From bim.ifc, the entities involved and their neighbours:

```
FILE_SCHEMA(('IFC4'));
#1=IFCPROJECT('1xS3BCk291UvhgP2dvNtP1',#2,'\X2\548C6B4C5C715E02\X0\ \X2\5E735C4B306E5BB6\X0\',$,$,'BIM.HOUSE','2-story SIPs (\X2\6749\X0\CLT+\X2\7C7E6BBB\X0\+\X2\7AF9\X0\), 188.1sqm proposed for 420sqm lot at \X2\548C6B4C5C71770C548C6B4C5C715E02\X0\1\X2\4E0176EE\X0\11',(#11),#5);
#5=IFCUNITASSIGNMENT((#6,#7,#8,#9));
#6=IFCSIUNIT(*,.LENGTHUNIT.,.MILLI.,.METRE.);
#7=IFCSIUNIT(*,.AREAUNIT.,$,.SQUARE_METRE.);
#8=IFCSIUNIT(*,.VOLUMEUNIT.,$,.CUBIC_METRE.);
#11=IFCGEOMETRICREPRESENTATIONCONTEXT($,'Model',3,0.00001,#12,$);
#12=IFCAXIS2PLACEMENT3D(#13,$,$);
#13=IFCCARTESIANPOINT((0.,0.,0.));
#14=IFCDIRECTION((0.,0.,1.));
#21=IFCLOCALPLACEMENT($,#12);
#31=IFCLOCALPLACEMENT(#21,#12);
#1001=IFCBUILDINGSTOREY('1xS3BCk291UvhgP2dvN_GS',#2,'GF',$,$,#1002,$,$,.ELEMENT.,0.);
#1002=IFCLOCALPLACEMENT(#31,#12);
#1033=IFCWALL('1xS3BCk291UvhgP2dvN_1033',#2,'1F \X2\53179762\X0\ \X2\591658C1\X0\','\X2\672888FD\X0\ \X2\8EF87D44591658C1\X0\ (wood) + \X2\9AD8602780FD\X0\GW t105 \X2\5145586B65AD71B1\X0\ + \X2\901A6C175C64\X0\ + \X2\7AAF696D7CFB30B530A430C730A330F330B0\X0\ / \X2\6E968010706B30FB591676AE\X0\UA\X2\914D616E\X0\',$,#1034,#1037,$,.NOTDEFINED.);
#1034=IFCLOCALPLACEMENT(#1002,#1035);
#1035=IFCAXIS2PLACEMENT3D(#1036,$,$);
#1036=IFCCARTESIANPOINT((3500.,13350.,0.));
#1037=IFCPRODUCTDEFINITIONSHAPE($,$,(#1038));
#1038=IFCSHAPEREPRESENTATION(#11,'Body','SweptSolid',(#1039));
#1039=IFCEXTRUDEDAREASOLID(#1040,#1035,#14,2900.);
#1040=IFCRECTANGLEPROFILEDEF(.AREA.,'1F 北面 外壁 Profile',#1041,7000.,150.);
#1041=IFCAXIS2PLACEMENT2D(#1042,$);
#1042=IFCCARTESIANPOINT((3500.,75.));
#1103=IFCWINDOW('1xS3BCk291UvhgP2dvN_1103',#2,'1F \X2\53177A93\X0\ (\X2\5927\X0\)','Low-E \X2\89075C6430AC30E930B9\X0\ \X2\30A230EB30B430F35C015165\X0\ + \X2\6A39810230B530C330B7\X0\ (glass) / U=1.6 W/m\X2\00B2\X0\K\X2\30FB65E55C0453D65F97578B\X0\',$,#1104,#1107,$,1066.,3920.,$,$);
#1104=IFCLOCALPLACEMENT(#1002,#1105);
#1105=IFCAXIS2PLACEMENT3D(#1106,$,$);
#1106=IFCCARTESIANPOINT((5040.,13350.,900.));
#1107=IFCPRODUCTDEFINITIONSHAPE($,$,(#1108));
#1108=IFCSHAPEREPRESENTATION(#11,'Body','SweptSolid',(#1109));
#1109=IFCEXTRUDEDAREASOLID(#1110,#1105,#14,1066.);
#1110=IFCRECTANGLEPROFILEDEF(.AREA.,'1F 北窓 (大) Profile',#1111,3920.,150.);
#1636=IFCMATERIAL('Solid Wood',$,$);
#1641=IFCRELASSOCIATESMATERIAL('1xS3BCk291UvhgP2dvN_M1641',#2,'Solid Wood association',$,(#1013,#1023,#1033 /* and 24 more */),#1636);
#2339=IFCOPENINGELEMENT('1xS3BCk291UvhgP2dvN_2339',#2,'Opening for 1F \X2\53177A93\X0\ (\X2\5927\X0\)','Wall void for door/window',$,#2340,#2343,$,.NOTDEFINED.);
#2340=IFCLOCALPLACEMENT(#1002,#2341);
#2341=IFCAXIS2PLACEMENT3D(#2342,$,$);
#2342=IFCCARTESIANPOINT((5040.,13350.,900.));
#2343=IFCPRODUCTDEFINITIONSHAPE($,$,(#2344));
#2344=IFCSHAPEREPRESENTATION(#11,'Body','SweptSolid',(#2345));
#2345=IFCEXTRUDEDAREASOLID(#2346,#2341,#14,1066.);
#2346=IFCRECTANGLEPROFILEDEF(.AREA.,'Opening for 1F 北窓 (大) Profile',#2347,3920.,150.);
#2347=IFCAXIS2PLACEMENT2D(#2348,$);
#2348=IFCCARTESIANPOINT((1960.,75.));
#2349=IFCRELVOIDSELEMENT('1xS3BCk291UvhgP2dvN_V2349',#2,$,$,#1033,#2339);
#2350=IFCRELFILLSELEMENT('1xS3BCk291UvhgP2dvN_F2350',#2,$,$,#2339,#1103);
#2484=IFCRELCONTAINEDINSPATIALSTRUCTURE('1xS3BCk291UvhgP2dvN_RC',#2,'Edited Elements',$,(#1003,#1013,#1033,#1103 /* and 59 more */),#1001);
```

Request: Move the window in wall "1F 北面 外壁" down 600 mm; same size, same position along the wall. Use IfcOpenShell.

```python
import numpy as np
import ifcopenshell
import ifcopenshell.api.geometry
import ifcopenshell.util.placement
import ifcopenshell.util.unit

model = ifcopenshell.open("bim.ifc")
unit_scale = ifcopenshell.util.unit.calculate_unit_scale(model)

window = model.by_guid("1xS3BCk291UvhgP2dvN_1103")
opening = window.FillsVoids[0].RelatingOpeningElement
dz = -0.6 / unit_scale

shift = np.array([0.0, 0.0, dz])
# The window is not placed relative to its opening, so move both.
for product in (opening, window):
    matrix = ifcopenshell.util.placement.get_local_placement(product.ObjectPlacement)
    matrix[:3, 3] += shift
    ifcopenshell.api.geometry.edit_object_placement(model, product=product, matrix=matrix, is_si=False)

print(f"moved by {dz * unit_scale:+.3f} m")

model.write("bim_updated.ifc")
```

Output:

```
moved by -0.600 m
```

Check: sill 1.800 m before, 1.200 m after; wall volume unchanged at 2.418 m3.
